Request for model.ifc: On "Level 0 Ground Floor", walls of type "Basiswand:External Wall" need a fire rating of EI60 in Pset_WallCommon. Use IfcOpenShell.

First a look at what the model holds.

```python
import ifcopenshell
import ifcopenshell.util.element

model = ifcopenshell.open("model.ifc")
print(model.schema)
storey = next(s for s in model.by_type("IfcBuildingStorey") if s.Name == "Level 0 Ground Floor")
walls = [e for e in ifcopenshell.util.element.get_decomposition(storey) if e.is_a("IfcWall")]
seen = {}
for e in walls:
    element_type = ifcopenshell.util.element.get_type(e)
    key = (element_type.Name if element_type != e and element_type else None, ifcopenshell.util.element.get_pset(e, "Pset_WallCommon", "FireRating"))
    seen[key] = seen.get(key, 0) + 1
for (name, value), count in sorted(seen.items(), key=str):
    print(count, "x", name, "|", value)
```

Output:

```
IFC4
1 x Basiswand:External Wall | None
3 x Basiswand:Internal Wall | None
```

```python
import ifcopenshell
import ifcopenshell.api.pset
import ifcopenshell.util.element

model = ifcopenshell.open("model.ifc")

storey = next(s for s in model.by_type("IfcBuildingStorey") if s.Name == "Level 0 Ground Floor")
walls = [e for e in ifcopenshell.util.element.get_decomposition(storey) if e.is_a("IfcWall")]

count = 0
for e in walls:
    element_type = ifcopenshell.util.element.get_type(e)
    if element_type in (None, e) or element_type.Name != "Basiswand:External Wall":
        continue
    # add_pset returns the element's existing set when there is one.
    pset = ifcopenshell.api.pset.add_pset(model, product=e, name="Pset_WallCommon")
    ifcopenshell.api.pset.edit_pset(model, pset=pset, properties={"FireRating": "EI60"})
    count += 1

print(count, "walls updated")

model.write("model-out.ifc")
```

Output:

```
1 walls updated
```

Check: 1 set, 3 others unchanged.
